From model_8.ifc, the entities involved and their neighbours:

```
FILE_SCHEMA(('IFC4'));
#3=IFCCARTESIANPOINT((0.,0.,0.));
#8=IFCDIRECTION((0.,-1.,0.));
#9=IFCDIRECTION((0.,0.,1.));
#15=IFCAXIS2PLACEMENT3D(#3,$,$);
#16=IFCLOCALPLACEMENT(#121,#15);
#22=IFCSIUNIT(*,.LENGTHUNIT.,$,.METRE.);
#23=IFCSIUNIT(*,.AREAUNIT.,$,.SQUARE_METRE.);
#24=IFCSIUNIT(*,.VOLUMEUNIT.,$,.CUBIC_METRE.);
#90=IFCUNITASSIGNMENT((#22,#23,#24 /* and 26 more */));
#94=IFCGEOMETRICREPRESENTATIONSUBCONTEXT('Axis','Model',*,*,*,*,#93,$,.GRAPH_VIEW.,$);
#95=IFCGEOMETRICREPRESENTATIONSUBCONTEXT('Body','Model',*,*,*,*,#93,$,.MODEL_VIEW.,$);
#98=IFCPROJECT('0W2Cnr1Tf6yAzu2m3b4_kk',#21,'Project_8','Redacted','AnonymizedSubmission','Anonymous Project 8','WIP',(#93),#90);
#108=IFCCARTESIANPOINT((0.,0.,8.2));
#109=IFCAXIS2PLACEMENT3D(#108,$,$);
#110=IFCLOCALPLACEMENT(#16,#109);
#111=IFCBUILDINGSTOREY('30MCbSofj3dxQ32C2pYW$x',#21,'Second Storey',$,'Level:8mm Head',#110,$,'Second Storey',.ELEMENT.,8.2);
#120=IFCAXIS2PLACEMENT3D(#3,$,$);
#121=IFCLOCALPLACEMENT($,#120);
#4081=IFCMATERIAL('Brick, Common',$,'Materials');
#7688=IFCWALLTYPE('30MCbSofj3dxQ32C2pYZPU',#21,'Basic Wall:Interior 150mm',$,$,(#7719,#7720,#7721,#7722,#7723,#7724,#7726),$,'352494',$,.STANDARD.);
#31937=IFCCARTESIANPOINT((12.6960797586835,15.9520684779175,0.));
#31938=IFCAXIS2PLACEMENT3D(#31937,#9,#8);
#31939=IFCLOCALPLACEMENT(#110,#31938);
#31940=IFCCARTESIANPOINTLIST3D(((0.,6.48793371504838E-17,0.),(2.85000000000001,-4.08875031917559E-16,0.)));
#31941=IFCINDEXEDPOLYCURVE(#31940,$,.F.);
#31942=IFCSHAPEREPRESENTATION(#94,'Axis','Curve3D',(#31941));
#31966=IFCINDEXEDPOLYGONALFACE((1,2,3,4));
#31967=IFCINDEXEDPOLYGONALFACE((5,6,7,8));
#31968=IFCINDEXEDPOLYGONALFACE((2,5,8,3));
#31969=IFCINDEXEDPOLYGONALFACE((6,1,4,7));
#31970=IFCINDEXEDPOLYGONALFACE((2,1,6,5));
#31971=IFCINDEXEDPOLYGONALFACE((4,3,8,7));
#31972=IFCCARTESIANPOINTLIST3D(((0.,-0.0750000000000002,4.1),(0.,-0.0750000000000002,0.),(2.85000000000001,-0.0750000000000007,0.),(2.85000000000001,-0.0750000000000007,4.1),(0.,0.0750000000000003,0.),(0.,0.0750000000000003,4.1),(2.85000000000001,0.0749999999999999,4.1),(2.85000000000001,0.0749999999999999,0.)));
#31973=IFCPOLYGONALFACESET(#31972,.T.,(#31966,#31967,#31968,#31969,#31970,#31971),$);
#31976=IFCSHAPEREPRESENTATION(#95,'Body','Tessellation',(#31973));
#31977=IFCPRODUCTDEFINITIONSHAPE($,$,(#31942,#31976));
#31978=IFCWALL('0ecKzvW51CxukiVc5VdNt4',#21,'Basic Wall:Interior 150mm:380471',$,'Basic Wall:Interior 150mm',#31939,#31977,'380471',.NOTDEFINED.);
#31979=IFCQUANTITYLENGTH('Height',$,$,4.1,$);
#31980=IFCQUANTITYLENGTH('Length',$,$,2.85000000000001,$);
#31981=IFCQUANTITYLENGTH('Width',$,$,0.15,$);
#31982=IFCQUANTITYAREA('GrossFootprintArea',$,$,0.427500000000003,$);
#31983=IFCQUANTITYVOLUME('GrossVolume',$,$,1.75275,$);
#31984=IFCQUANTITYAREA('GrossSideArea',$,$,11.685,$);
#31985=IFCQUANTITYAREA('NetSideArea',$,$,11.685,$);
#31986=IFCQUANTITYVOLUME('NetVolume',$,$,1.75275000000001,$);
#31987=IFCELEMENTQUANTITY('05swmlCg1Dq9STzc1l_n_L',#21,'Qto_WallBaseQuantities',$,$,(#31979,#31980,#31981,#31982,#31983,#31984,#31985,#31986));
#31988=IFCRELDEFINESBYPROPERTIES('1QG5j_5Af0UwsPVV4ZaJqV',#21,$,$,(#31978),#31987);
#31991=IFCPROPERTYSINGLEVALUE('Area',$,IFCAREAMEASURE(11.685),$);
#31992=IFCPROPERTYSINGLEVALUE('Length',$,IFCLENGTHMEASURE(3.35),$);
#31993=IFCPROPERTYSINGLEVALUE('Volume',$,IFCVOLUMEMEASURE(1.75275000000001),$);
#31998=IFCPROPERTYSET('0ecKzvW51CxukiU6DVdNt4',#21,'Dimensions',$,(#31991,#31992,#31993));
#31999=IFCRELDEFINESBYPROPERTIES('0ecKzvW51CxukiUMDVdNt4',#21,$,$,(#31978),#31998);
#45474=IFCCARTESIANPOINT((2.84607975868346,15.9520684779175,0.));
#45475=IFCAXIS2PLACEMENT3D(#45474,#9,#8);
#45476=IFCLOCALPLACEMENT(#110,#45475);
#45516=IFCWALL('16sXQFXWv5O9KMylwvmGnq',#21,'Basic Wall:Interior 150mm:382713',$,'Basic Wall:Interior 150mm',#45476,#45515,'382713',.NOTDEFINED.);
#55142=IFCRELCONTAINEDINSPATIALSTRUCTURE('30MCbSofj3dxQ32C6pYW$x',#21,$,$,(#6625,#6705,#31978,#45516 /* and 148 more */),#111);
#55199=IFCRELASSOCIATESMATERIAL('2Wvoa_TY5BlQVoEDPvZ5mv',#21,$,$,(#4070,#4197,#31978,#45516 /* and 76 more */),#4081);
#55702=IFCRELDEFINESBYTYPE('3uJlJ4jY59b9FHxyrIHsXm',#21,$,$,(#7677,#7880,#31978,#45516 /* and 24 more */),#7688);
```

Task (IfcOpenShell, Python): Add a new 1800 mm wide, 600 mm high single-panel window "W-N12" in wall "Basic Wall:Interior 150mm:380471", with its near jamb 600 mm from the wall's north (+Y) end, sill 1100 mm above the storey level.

```python
import numpy as np
import ifcopenshell
import ifcopenshell.api.feature
import ifcopenshell.api.geometry
import ifcopenshell.api.pset
import ifcopenshell.api.root
import ifcopenshell.api.spatial
import ifcopenshell.geom
import ifcopenshell.util.element
import ifcopenshell.util.placement
import ifcopenshell.util.representation
import ifcopenshell.util.shape
import ifcopenshell.util.unit

model = ifcopenshell.open("model_8.ifc")
unit_scale = ifcopenshell.util.unit.calculate_unit_scale(model)
area_scale = ifcopenshell.util.unit.calculate_unit_scale(model, "AREAUNIT")
volume_scale = ifcopenshell.util.unit.calculate_unit_scale(model, "VOLUMEUNIT")
settings = ifcopenshell.geom.settings()


def volume(element):
    """Net volume in cubic metres, openings subtracted."""
    shape = ifcopenshell.geom.create_shape(settings, element)
    return ifcopenshell.util.shape.get_volume(shape.geometry)


wall = model.by_guid("0ecKzvW51CxukiVc5VdNt4")
storey = ifcopenshell.util.element.get_container(wall, ifc_class="IfcBuildingStorey")
context = ifcopenshell.util.representation.get_context(model, "Model", "Body", "MODEL_VIEW")
before = volume(wall)

width, height, from_end, sill = 1.8, 0.6, 0.6, 1.1  # metres

# The wall runs along its own X axis, and the end named is its -X end.
wall_shape = ifcopenshell.geom.create_shape(settings, wall)
x, y, z = ifcopenshell.util.shape.get_vertices(wall_shape.geometry).T
start = x.min() + from_end
face, thickness = float(y.min()), float(y.max() - y.min())
wall_matrix = ifcopenshell.util.placement.get_local_placement(wall.ObjectPlacement)
level = ifcopenshell.util.placement.get_local_placement(storey.ObjectPlacement)[2, 3]


def in_wall(x, y):
    """Placement at x, y metres in the wall's axes, at sill height."""
    matrix = wall_matrix.copy()
    matrix[:, 3] = wall_matrix @ np.array([x / unit_scale, y / unit_scale, 0.0, 1.0])
    matrix[2, 3] = level + sill / unit_scale
    return matrix


# Opening: a box that overshoots both wall faces by 50 mm.
opening = ifcopenshell.api.root.create_entity(model, ifc_class="IfcOpeningElement", predefined_type="OPENING")
box = ifcopenshell.api.geometry.add_wall_representation(
    model, context=context, length=width, height=height, thickness=thickness + 0.1
)
ifcopenshell.api.geometry.assign_representation(model, product=opening, representation=box)
ifcopenshell.api.geometry.edit_object_placement(model, product=opening, matrix=in_wall(start, face - 0.05), is_si=False)
ifcopenshell.api.feature.add_feature(model, feature=opening, element=wall)

window = ifcopenshell.api.root.create_entity(model, ifc_class="IfcWindow", name="W-N12", predefined_type="WINDOW")
window.OverallWidth, window.OverallHeight = width / unit_scale, height / unit_scale
window.PartitioningType = "SINGLE_PANEL"
body = ifcopenshell.api.geometry.add_window_representation(
    model,
    context=context,
    overall_width=window.OverallWidth,
    overall_height=window.OverallHeight,
    partition_type="SINGLE_PANEL",
)
ifcopenshell.api.geometry.assign_representation(model, product=window, representation=body)
ifcopenshell.api.spatial.assign_container(model, products=[window], relating_structure=storey)
ifcopenshell.api.feature.add_filling(model, opening=opening, element=window)

# Centre the window in the wall's thickness.
ifcopenshell.api.geometry.edit_object_placement(model, product=window, matrix=in_wall(start, face), is_si=False)
window_shape = ifcopenshell.geom.create_shape(settings, window)
depth = ifcopenshell.util.shape.get_vertices(window_shape.geometry)[:, 1]
offset = face + thickness / 2 - (depth.min() + depth.max()) / 2
ifcopenshell.api.geometry.edit_object_placement(model, product=window, matrix=in_wall(start, offset), is_si=False)

after = volume(wall)

# Update the wall's stored quantities.
qto = model.by_id(ifcopenshell.util.element.get_pset(wall, "Qto_WallBaseQuantities", should_inherit=False)["id"])
ifcopenshell.api.pset.edit_qto(model, qto=qto, properties={
    "NetSideArea": after / thickness / area_scale,
    "NetVolume": after / volume_scale,
})
pset = model.by_id(ifcopenshell.util.element.get_pset(wall, "Dimensions", should_inherit=False)["id"])
ifcopenshell.api.pset.edit_pset(model, pset=pset, properties={
    "Area": model.create_entity("IfcAreaMeasure", after / thickness / area_scale),
    "Volume": model.create_entity("IfcVolumeMeasure", after / volume_scale),
})

print(f"wall volume {before:.3f} -> {after:.3f} m3")

model.write("model_8_v2.ifc")
```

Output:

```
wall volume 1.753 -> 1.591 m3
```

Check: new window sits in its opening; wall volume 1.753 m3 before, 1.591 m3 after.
